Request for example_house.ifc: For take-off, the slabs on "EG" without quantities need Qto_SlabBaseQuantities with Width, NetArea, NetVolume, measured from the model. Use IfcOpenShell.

First a look at what the model holds.

```python
import ifcopenshell
import ifcopenshell.util.element
import ifcopenshell.util.unit

model = ifcopenshell.open("example_house.ifc")
print(model.schema)
for unit_type in ("LENGTHUNIT", "AREAUNIT", "VOLUMEUNIT"):
    print(unit_type, ifcopenshell.util.unit.calculate_unit_scale(model, unit_type))
storey = next(s for s in model.by_type("IfcBuildingStorey") if s.Name == "EG")
slabs = [e for e in ifcopenshell.util.element.get_decomposition(storey) if e.is_a("IfcSlab")]
for e in sorted(slabs, key=lambda e: e.id()):
    print(e.id(), e.is_a(), e.Name, list(ifcopenshell.util.element.get_psets(e, qtos_only=True)), sep=" | ")
```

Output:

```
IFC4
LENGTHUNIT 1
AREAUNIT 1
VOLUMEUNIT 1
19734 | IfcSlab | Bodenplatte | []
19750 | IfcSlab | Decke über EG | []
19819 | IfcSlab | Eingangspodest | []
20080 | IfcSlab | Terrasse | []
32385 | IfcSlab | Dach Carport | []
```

```python
import ifcopenshell
import ifcopenshell.api.pset
import ifcopenshell.geom
import ifcopenshell.util.element
import ifcopenshell.util.shape
import ifcopenshell.util.unit

model = ifcopenshell.open("example_house.ifc")
unit_scale = ifcopenshell.util.unit.calculate_unit_scale(model)
area_scale = ifcopenshell.util.unit.calculate_unit_scale(model, "AREAUNIT")
volume_scale = ifcopenshell.util.unit.calculate_unit_scale(model, "VOLUMEUNIT")
settings = ifcopenshell.geom.settings()

storey = next(s for s in model.by_type("IfcBuildingStorey") if s.Name == "EG")
slabs = [e for e in ifcopenshell.util.element.get_decomposition(storey) if e.is_a("IfcSlab")]

for e in sorted(slabs, key=lambda e: e.id()):
    if ifcopenshell.util.element.get_psets(e, qtos_only=True, should_inherit=False):
        continue
    # Geometry comes back in metres, in the element's own axes.
    shape = ifcopenshell.geom.create_shape(settings, e)
    values = {
        "Width": ifcopenshell.util.shape.get_z(shape.geometry) / unit_scale,
        "NetArea": ifcopenshell.util.shape.get_footprint_area(shape.geometry) / area_scale,
        "NetVolume": ifcopenshell.util.shape.get_volume(shape.geometry) / volume_scale,
    }
    qto = ifcopenshell.api.pset.add_qto(model, product=e, name="Qto_SlabBaseQuantities")
    ifcopenshell.api.pset.edit_qto(model, qto=qto, properties=values)
    print(e.id(), {k: round(v, 3) for k, v in values.items()})

model.write("example_house_edited.ifc")
```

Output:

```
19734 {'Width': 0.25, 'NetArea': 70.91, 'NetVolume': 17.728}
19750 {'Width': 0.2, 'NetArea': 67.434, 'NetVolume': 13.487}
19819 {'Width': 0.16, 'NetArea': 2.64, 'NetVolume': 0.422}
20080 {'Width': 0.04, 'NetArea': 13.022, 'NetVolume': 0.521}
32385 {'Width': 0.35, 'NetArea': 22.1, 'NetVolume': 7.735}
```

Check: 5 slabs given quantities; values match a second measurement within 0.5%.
